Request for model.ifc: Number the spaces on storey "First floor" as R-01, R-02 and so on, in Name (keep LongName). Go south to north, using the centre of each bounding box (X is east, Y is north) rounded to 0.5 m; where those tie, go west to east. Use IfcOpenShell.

First a look at what the model holds.

```python
import ifcopenshell
import ifcopenshell.util.element
import ifcopenshell.util.placement

model = ifcopenshell.open("model.ifc")
print(model.schema)
storey = next(s for s in model.by_type("IfcBuildingStorey") if s.Name == "First floor")
spaces = [e for e in ifcopenshell.util.element.get_decomposition(storey) if e.is_a("IfcSpace")]
for e in sorted(spaces, key=lambda e: e.id()):
    origin = ifcopenshell.util.placement.get_local_placement(e.ObjectPlacement)[:3, 3]
    print(e.id(), e.Name, e.LongName, origin.round(2) + 0.0, sep=" | ")
```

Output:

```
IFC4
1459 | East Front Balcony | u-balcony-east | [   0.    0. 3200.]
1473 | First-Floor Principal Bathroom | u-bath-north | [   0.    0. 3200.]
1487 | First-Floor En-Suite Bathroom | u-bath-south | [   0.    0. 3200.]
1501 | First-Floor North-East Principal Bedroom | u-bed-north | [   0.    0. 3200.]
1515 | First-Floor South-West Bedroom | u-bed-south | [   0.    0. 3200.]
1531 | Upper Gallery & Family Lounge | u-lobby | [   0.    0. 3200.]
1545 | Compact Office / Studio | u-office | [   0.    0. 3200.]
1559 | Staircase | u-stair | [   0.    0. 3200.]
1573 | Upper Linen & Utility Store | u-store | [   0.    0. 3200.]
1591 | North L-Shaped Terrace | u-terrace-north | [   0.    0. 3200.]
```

```python
import ifcopenshell
import ifcopenshell.geom
import ifcopenshell.util.element
import ifcopenshell.util.shape

model = ifcopenshell.open("model.ifc")
settings = ifcopenshell.geom.settings()
settings.set("use-world-coords", True)


def centre(element):
    shape = ifcopenshell.geom.create_shape(settings, element)
    return ifcopenshell.util.shape.get_bbox_centroid(shape.geometry)


storey = next(s for s in model.by_type("IfcBuildingStorey") if s.Name == "First floor")
spaces = [e for e in ifcopenshell.util.element.get_decomposition(storey) if e.is_a("IfcSpace")]

# Insertion points can sit at a corner or the storey origin, so sort by the geometry (in metres).
centres = {e: centre(e) for e in spaces}
spaces.sort(key=lambda e: (round(centres[e][1] / 0.5), centres[e][0]))

for i, e in enumerate(spaces, start=1):
    number = f"R-{i:02d}"
    e.Name = number
    print(e.id(), number)

model.write("model_updated.ifc")
```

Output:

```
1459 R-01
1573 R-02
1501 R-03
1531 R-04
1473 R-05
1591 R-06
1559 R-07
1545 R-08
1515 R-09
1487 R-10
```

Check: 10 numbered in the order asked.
